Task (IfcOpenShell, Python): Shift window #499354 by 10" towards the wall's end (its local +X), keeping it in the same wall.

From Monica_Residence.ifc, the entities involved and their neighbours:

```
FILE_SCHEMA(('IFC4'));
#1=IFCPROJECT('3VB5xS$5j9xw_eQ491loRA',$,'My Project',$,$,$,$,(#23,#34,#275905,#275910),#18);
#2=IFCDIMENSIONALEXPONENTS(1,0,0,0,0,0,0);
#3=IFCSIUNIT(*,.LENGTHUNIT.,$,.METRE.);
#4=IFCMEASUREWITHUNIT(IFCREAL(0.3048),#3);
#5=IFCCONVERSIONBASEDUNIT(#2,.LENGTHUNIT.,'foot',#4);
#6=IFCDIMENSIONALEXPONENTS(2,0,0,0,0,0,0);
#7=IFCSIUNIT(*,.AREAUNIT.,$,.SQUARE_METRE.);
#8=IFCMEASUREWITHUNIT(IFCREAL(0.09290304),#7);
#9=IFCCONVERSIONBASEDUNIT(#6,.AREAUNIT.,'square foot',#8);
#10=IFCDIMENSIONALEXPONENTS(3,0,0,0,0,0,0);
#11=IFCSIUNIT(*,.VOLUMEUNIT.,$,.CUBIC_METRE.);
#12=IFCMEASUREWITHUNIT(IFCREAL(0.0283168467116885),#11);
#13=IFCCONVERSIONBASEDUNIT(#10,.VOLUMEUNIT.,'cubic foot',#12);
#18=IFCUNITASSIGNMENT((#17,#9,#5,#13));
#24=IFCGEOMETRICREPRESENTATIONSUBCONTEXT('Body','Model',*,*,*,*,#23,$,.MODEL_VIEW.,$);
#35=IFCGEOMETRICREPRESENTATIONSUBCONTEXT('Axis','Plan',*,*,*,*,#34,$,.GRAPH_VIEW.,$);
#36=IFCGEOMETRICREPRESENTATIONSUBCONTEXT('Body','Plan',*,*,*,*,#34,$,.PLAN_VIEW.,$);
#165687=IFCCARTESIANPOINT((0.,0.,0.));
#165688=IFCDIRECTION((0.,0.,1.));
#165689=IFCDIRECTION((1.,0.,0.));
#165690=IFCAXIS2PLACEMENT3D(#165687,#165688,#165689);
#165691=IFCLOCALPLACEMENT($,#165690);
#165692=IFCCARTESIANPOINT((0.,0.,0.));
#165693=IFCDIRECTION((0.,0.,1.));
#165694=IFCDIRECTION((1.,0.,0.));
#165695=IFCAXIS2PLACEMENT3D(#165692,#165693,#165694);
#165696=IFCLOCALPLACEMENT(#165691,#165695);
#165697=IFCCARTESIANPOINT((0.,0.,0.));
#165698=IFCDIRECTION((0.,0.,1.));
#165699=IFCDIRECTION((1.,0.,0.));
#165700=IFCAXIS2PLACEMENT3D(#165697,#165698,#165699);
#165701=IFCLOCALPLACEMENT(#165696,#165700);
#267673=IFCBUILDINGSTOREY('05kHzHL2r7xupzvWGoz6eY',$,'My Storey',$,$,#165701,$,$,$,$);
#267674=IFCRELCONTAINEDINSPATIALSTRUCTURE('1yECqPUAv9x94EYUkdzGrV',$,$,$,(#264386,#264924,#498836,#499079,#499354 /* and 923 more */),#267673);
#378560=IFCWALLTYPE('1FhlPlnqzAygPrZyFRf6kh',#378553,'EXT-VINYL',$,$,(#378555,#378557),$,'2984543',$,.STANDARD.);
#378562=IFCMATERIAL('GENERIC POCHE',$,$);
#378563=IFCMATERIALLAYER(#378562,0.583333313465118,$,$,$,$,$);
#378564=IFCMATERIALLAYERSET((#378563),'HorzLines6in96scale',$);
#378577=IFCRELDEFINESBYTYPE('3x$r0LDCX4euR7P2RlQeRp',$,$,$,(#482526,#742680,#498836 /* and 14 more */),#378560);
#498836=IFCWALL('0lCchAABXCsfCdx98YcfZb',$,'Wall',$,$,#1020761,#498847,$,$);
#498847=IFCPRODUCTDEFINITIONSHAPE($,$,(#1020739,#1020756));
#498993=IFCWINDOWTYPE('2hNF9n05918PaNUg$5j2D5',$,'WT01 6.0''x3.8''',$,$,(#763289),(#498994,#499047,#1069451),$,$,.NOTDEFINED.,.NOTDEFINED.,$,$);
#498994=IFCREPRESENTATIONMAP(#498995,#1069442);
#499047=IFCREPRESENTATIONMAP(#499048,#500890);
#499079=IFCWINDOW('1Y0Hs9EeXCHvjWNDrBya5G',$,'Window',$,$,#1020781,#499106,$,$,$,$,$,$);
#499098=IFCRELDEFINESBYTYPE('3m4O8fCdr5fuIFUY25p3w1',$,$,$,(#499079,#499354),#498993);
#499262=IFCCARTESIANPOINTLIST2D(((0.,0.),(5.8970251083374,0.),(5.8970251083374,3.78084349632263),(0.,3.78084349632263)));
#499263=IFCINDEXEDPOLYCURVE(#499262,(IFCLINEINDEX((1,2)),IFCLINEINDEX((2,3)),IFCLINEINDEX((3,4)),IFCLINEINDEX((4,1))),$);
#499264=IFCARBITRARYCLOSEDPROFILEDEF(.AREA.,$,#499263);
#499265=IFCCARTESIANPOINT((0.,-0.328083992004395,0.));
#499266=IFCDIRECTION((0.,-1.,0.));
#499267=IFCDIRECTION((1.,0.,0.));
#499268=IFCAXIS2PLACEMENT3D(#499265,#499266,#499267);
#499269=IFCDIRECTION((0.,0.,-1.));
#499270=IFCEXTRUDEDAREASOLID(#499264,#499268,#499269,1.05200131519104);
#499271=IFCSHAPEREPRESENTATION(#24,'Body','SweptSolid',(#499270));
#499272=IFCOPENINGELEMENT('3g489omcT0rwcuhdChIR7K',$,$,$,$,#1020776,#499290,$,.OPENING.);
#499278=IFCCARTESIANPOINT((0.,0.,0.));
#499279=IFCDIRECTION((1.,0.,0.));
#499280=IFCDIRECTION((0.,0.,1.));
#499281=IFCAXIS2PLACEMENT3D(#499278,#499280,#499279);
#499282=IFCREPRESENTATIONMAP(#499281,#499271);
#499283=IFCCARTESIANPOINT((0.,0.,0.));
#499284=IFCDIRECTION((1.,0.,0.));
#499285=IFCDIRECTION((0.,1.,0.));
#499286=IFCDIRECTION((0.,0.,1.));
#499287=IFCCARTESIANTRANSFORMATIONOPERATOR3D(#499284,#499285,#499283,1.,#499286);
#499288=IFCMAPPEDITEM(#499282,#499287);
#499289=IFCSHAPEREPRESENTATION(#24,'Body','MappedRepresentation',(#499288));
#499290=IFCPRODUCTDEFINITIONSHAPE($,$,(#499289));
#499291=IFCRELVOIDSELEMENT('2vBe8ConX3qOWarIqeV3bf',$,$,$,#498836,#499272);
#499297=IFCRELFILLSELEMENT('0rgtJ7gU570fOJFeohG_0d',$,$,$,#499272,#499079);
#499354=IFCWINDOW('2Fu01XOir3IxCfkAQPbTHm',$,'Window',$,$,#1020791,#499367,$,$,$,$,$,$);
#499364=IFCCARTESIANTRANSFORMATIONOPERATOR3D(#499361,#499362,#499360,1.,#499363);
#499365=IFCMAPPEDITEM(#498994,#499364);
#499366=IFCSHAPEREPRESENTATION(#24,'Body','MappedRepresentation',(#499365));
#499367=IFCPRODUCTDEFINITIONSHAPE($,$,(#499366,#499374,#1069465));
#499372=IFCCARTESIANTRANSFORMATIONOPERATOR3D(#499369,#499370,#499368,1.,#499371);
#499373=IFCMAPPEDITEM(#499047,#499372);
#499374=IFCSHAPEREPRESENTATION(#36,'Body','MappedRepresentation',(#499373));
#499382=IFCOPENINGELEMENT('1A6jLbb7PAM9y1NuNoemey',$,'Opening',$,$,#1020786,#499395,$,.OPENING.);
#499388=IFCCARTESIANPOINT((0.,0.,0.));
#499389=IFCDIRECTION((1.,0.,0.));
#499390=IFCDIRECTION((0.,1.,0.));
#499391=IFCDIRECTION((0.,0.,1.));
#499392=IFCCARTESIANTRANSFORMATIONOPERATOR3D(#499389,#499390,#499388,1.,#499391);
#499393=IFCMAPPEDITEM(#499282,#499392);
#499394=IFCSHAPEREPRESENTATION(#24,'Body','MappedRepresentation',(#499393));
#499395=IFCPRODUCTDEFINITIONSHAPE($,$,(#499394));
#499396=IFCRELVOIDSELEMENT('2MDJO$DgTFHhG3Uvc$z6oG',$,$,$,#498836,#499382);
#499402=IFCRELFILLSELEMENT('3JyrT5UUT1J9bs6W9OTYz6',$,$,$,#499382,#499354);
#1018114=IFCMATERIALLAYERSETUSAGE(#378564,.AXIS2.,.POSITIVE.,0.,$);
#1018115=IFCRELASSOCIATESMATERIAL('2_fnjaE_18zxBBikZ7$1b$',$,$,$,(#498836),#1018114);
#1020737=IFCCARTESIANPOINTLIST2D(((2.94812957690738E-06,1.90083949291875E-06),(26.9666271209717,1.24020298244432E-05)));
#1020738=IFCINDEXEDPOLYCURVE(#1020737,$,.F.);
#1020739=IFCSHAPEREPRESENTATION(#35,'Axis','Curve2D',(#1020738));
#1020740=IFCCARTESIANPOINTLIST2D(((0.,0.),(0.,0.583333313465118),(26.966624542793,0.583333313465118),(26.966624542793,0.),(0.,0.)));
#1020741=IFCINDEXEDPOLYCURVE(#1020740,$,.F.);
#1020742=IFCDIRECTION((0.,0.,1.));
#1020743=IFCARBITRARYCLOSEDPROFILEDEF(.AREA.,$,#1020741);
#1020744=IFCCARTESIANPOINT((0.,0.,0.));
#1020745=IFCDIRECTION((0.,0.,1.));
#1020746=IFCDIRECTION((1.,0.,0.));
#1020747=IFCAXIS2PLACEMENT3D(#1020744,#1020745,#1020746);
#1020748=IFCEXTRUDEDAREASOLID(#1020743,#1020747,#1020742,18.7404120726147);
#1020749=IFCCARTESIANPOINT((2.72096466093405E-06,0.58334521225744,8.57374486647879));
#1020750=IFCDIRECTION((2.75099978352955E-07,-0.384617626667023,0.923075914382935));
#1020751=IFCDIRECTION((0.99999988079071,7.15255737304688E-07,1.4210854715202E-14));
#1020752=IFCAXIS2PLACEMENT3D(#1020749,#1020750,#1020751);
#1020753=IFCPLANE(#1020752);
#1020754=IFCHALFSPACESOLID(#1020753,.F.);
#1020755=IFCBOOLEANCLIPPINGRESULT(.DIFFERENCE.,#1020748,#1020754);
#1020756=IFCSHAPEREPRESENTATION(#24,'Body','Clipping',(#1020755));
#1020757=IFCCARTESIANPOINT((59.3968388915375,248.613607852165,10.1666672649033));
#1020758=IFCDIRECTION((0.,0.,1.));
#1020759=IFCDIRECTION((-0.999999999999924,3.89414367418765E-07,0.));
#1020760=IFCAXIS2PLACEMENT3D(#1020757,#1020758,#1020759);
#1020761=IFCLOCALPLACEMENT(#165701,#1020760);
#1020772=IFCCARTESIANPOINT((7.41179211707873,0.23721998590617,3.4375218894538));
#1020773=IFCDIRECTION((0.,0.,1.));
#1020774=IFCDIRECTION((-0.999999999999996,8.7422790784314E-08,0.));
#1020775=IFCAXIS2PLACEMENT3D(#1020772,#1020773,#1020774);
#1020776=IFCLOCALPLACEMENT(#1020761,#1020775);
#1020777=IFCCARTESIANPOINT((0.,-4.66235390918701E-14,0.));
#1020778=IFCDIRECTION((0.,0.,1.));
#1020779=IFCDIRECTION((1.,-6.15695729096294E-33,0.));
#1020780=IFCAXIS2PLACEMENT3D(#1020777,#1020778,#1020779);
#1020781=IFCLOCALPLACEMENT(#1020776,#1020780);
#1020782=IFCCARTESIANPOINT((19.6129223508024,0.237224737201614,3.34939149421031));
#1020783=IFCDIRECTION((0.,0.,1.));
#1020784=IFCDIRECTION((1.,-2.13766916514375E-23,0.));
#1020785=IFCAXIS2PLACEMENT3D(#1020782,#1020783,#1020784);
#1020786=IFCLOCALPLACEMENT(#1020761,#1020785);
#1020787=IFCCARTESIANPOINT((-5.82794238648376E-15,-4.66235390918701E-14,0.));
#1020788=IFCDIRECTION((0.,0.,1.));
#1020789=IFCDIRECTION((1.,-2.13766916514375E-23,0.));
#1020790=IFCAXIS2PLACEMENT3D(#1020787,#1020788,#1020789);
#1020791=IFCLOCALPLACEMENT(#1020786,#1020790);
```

```python
import ifcopenshell
import ifcopenshell.api.geometry
import ifcopenshell.util.placement
import ifcopenshell.util.unit

model = ifcopenshell.open("Monica_Residence.ifc")
unit_scale = ifcopenshell.util.unit.calculate_unit_scale(model)

window = model.by_guid("2Fu01XOir3IxCfkAQPbTHm")
opening = window.FillsVoids[0].RelatingOpeningElement
wall = opening.VoidsElements[0].RelatingBuildingElement

wall_matrix = ifcopenshell.util.placement.get_local_placement(wall.ObjectPlacement)
shift = wall_matrix[:3, 0] * 10 * 0.0254 / unit_scale
before = ifcopenshell.util.placement.get_local_placement(window.ObjectPlacement)[:3, 3].copy()

# The window is placed relative to its opening, so it follows when the opening moves.
matrix = ifcopenshell.util.placement.get_local_placement(opening.ObjectPlacement)
matrix[:3, 3] += shift
ifcopenshell.api.geometry.edit_object_placement(
    model, product=opening, matrix=matrix, is_si=False, should_transform_children=True
)

after = ifcopenshell.util.placement.get_local_placement(window.ObjectPlacement)[:3, 3]
print("window moved by", (after - before).round(3) + 0.0)

model.write("Monica_Residence-out.ifc")
```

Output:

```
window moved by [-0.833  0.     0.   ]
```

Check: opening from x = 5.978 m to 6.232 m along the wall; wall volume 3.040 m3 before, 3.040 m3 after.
